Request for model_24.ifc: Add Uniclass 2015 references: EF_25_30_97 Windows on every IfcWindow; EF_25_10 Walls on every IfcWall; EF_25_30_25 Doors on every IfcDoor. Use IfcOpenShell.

First a look at what the model holds.

```python
import ifcopenshell

model = ifcopenshell.open("model_24.ifc")
print(model.schema)
print("classifications:", [c.Name for c in model.by_type("IfcClassification")])
for ifc_class in ("IfcDoor", "IfcRoof", "IfcStair", "IfcWall", "IfcWindow"):
    print(ifc_class, len(model.by_type(ifc_class)))
```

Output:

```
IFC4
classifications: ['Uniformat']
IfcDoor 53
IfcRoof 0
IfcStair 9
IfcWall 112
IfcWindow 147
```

```python
import ifcopenshell
import ifcopenshell.api.classification

model = ifcopenshell.open("model_24.ifc")

system = ifcopenshell.api.classification.add_classification(model, classification="Uniclass 2015")

codes = {
    "IfcWindow": ("EF_25_30_97", "Windows"),
    "IfcWall": ("EF_25_10", "Walls"),
    "IfcDoor": ("EF_25_30_25", "Doors"),
}
for ifc_class, (code, name) in codes.items():
    products = model.by_type(ifc_class)
    ifcopenshell.api.classification.add_reference(
        model, products=products, classification=system, identification=code, name=name
    )
    print(code, len(products))

model.write("model_24_updated.ifc")
```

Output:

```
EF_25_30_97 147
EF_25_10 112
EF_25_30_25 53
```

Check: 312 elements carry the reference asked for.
